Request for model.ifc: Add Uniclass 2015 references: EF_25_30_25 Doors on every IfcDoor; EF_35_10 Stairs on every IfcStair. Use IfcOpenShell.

First a look at what the model holds.

```python
import ifcopenshell

model = ifcopenshell.open("model.ifc")
print(model.schema)
print("classifications:", [c.Name for c in model.by_type("IfcClassification")])
for ifc_class in ("IfcDoor", "IfcRoof", "IfcStair", "IfcWall", "IfcWindow"):
    print(ifc_class, len(model.by_type(ifc_class)))
```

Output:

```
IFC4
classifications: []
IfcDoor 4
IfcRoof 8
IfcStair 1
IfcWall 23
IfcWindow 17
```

```python
import ifcopenshell
import ifcopenshell.api.classification

model = ifcopenshell.open("model.ifc")

system = ifcopenshell.api.classification.add_classification(model, classification="Uniclass 2015")

codes = {
    "IfcDoor": ("EF_25_30_25", "Doors"),
    "IfcStair": ("EF_35_10", "Stairs"),
}
for ifc_class, (code, name) in codes.items():
    products = model.by_type(ifc_class)
    ifcopenshell.api.classification.add_reference(
        model, products=products, classification=system, identification=code, name=name
    )
    print(code, len(products))

model.write("model_rev.ifc")
```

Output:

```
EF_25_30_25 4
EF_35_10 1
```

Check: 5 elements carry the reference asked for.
